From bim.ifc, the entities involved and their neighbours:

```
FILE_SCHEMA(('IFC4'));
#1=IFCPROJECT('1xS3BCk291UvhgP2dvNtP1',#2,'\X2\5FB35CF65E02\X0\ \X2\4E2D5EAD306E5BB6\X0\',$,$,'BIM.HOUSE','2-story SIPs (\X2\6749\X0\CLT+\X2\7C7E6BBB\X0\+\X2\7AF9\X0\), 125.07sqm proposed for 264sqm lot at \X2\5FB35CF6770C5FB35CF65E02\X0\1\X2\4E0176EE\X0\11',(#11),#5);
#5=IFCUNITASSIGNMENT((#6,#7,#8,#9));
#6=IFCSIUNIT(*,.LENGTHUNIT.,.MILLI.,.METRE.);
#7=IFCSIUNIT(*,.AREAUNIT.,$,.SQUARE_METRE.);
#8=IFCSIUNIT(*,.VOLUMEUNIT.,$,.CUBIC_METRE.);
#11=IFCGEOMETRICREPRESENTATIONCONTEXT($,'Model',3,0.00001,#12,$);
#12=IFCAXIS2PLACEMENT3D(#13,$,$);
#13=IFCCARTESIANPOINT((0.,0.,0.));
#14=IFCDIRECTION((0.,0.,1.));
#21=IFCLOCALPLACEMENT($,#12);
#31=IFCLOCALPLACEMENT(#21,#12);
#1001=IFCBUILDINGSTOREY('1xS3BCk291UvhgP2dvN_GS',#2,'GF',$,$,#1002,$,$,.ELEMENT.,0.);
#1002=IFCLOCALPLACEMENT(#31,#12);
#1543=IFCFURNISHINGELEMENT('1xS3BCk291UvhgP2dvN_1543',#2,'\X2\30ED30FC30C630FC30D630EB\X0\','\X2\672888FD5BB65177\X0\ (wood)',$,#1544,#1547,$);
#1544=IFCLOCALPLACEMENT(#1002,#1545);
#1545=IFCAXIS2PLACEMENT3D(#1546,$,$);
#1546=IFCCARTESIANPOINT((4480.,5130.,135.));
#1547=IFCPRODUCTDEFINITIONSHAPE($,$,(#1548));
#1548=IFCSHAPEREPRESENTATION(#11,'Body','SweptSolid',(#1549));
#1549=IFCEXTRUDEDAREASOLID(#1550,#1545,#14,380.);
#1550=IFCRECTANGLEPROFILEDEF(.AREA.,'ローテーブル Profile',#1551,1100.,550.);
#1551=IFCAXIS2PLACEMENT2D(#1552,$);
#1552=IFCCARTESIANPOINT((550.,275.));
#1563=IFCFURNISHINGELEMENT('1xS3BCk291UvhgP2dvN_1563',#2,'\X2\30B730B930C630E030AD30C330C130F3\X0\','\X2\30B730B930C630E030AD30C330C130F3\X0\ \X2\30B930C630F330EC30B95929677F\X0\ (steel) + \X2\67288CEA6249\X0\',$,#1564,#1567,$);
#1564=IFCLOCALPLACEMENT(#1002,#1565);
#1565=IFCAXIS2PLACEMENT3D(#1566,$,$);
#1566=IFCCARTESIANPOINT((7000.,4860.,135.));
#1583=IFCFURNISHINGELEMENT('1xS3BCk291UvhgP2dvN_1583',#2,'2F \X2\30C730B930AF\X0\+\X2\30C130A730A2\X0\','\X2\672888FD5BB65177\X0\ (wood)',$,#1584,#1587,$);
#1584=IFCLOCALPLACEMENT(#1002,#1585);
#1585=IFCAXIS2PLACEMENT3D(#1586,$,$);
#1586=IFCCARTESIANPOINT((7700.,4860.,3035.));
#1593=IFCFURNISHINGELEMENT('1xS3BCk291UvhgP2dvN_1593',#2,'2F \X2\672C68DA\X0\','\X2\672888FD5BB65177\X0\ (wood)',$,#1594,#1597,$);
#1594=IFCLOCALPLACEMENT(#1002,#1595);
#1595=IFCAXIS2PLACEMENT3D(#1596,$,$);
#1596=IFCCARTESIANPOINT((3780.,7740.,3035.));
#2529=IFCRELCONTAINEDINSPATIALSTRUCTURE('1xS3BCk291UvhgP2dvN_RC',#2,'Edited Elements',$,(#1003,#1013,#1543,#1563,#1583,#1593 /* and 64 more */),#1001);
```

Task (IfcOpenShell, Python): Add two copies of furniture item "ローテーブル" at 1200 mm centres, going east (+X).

```python
import numpy as np
import ifcopenshell
import ifcopenshell.api.geometry
import ifcopenshell.api.root
import ifcopenshell.util.element
import ifcopenshell.util.placement

model = ifcopenshell.open("bim.ifc")


def reuse_history(source, copy):
    """copy_class also copies each property set's owner history, people and application; keep the originals."""
    for rel in copy.IsDefinedBy:
        if rel.is_a("IfcRelDefinesByProperties") and (history := rel.RelatingPropertyDefinition.OwnerHistory):
            rel.RelatingPropertyDefinition.OwnerHistory = source.OwnerHistory
            ifcopenshell.util.element.remove_deep2(model, history)


source = model.by_guid("1xS3BCk291UvhgP2dvN_1543")
base = ifcopenshell.util.placement.get_local_placement(source.ObjectPlacement)
step = np.array([1.0, 0.0, 0.0]) * 1200.0

for i in range(1, 3):
    copy = ifcopenshell.api.root.copy_class(model, product=source)
    copy.Representation = ifcopenshell.util.element.copy_deep(
        model, source.Representation, exclude=["IfcGeometricRepresentationContext", "IfcRepresentationMap"]
    )
    reuse_history(source, copy)
    matrix = base.copy()
    matrix[:3, 3] += i * step
    print("added at", matrix[:3, 3].round(3) + 0.0)
    ifcopenshell.api.geometry.edit_object_placement(model, product=copy, matrix=matrix, is_si=False)

model.write("bim_v2.ifc")
```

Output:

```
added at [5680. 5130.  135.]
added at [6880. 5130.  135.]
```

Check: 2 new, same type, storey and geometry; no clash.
